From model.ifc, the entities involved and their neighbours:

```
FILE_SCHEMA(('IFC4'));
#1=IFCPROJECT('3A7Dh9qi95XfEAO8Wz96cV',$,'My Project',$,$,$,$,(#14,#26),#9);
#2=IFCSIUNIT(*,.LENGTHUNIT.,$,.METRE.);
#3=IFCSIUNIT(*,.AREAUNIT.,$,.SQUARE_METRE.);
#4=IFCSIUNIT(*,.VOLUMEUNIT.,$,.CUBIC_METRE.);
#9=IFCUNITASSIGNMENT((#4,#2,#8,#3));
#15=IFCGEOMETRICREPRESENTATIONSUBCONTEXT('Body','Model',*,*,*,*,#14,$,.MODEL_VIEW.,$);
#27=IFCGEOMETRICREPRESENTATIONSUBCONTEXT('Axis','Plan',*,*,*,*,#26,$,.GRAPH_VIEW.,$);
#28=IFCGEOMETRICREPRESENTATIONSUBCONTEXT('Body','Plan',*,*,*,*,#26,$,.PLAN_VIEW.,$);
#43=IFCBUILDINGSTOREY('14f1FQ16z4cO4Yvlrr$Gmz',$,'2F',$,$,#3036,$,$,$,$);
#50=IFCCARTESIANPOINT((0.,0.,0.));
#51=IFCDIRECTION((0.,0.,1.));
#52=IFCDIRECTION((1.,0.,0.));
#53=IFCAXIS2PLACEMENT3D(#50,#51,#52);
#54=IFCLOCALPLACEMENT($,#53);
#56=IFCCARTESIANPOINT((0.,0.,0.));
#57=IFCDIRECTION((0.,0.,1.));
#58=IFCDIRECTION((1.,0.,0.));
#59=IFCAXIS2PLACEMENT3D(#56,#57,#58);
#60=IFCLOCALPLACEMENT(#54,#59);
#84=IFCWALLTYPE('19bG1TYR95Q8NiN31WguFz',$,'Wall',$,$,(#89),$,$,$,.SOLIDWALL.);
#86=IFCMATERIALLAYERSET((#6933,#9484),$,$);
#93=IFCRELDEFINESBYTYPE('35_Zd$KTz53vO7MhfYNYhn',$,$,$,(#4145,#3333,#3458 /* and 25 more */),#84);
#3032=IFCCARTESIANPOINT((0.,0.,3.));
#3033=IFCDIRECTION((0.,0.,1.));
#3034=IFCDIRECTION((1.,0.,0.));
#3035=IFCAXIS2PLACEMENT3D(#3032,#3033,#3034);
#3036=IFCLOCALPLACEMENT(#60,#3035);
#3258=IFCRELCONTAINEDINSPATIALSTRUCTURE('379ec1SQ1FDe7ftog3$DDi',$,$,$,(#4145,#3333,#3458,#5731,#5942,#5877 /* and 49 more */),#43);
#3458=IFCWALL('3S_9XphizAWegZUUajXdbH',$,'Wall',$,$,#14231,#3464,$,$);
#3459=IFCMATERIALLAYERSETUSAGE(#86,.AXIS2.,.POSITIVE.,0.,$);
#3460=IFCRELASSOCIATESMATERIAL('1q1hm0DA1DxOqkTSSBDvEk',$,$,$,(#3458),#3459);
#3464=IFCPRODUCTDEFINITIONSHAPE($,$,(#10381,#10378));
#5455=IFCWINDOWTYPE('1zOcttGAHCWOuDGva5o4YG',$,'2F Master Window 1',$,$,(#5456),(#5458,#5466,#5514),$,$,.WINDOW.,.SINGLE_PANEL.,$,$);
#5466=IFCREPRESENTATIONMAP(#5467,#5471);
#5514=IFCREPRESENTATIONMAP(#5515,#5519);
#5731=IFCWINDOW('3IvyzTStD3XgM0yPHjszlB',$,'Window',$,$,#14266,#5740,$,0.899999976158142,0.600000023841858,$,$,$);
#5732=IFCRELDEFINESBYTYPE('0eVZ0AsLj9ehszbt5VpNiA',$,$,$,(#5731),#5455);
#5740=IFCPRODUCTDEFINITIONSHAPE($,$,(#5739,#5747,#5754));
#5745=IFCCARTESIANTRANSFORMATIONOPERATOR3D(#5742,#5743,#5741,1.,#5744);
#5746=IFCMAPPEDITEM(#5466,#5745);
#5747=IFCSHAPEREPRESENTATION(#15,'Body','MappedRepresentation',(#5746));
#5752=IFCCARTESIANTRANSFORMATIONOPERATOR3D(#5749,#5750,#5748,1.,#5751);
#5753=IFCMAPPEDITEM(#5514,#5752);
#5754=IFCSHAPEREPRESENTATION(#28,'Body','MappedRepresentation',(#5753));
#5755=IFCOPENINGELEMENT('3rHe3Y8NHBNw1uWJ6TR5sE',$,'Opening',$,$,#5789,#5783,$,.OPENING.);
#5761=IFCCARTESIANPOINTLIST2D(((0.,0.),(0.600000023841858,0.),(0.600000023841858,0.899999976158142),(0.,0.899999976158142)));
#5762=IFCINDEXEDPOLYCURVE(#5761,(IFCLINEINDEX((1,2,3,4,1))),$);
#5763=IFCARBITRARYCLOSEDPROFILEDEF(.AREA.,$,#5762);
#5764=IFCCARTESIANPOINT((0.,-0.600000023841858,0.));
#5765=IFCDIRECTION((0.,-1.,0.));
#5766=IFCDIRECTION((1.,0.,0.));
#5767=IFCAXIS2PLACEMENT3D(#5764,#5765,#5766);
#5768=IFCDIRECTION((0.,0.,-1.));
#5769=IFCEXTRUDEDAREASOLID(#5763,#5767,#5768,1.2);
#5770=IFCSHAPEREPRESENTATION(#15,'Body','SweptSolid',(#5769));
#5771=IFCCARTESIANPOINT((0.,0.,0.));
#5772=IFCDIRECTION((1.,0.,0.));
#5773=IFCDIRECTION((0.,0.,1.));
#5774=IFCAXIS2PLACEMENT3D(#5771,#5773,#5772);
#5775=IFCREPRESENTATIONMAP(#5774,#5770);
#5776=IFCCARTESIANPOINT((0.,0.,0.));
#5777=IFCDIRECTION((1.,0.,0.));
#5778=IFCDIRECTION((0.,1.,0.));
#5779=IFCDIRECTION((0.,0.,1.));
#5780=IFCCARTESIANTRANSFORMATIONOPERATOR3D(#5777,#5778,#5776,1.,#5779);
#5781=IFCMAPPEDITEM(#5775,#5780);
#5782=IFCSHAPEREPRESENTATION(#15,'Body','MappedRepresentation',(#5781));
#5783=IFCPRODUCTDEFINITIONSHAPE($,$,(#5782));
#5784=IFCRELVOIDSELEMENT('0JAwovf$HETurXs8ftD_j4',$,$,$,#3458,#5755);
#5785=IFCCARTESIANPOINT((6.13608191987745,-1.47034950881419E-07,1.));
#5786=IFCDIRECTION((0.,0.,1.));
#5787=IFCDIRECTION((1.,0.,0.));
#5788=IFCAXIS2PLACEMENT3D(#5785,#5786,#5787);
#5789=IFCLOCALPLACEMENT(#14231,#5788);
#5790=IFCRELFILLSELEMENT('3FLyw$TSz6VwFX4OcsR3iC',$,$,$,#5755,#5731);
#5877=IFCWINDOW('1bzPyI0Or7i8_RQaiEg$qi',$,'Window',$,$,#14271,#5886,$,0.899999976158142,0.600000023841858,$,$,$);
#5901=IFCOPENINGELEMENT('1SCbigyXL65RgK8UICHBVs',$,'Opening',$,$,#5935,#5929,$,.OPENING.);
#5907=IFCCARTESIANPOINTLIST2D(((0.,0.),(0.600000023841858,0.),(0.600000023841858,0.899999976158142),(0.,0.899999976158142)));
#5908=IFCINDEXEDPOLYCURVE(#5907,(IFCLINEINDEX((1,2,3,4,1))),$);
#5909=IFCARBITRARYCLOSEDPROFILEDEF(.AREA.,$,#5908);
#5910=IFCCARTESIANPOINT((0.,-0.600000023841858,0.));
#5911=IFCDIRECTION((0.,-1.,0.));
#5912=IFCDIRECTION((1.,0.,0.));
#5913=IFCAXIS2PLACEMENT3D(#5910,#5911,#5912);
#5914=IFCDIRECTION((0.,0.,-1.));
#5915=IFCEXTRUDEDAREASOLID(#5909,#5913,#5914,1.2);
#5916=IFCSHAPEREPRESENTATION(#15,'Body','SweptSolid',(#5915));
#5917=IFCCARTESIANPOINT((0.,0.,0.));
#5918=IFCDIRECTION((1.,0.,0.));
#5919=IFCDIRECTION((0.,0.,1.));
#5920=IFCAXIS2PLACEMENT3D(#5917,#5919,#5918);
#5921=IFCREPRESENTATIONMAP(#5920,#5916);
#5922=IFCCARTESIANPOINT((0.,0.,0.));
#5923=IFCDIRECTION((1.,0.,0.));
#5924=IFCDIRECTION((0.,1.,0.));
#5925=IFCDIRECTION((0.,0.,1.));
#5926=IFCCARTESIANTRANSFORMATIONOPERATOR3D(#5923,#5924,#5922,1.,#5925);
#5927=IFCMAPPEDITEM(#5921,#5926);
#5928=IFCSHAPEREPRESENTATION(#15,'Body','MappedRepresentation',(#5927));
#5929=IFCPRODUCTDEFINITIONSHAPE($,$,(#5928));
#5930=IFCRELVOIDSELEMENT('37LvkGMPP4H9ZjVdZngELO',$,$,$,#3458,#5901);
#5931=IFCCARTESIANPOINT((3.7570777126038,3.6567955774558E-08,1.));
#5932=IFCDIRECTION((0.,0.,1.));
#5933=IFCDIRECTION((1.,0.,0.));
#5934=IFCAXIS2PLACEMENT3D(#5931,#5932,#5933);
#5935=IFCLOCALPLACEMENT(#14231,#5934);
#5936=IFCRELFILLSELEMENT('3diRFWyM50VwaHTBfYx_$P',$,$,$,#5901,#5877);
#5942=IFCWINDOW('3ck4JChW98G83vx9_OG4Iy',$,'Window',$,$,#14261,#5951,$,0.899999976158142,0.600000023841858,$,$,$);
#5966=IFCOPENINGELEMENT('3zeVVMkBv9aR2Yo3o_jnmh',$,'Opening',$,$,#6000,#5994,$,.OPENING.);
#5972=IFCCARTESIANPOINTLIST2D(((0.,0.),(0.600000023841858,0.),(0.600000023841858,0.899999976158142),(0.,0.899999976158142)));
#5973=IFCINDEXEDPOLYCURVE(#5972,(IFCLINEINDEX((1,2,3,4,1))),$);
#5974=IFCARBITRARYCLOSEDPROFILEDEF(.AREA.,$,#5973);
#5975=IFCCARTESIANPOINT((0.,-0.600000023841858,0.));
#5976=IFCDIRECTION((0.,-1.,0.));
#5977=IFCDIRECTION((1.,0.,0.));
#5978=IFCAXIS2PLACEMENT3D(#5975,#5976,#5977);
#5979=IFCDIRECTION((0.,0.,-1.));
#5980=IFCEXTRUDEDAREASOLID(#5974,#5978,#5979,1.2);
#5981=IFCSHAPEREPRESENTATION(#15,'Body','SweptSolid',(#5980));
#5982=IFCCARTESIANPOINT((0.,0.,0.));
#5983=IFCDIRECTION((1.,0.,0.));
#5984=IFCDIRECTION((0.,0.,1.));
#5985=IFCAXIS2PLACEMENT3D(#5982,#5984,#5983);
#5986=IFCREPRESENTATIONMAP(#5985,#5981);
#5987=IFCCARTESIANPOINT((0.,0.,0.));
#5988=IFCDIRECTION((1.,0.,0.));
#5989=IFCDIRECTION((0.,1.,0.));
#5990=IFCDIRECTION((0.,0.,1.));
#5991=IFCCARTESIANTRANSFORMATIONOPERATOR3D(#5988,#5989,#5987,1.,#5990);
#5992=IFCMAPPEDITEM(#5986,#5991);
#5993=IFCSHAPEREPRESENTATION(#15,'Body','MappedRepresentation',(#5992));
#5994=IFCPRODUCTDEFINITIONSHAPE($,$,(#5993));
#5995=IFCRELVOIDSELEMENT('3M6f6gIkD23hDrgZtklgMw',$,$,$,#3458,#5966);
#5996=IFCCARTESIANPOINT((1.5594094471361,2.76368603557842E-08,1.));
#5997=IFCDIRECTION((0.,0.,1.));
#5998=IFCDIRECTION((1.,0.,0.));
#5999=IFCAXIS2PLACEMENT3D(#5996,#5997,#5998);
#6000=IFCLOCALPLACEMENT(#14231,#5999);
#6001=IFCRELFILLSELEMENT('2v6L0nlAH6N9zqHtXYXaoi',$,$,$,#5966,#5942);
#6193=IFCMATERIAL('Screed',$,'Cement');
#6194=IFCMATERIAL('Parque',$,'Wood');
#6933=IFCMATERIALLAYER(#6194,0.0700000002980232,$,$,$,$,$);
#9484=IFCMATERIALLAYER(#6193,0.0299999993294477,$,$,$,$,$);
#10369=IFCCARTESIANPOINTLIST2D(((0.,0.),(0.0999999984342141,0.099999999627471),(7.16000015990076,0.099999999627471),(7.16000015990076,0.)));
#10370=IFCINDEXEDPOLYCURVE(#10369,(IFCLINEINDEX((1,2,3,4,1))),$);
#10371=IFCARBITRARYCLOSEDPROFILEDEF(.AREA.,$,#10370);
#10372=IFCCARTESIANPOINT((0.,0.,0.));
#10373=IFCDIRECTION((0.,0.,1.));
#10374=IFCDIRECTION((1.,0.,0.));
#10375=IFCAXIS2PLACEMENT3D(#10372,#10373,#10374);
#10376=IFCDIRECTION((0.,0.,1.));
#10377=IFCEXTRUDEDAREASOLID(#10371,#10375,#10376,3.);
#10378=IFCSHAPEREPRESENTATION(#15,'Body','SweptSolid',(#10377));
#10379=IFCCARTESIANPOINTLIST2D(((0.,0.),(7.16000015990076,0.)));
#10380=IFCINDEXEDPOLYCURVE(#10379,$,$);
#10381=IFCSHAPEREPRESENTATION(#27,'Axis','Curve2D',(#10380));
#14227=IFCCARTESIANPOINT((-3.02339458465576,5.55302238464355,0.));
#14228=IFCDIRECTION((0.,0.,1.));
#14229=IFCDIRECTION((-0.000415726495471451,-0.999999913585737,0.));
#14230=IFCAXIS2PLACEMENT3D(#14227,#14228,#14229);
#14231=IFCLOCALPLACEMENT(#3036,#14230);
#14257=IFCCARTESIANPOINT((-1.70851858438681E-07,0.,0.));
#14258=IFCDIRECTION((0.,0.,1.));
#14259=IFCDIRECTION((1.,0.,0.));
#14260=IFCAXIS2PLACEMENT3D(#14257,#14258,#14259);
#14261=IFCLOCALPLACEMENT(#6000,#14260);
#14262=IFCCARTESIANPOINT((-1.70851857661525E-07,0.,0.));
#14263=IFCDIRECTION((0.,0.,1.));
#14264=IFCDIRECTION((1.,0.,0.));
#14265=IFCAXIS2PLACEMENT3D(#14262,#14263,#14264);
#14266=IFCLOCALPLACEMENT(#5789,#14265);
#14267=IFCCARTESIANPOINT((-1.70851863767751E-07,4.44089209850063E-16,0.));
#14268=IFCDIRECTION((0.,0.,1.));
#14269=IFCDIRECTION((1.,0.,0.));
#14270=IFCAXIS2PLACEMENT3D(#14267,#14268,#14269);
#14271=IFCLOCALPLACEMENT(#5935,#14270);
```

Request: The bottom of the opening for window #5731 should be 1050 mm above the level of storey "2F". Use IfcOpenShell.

```python
import numpy as np
import ifcopenshell
import ifcopenshell.api.geometry
import ifcopenshell.geom
import ifcopenshell.util.element
import ifcopenshell.util.placement
import ifcopenshell.util.shape
import ifcopenshell.util.unit

model = ifcopenshell.open("model.ifc")
unit_scale = ifcopenshell.util.unit.calculate_unit_scale(model)

window = model.by_guid("3IvyzTStD3XgM0yPHjszlB")
opening = window.FillsVoids[0].RelatingOpeningElement
storey = ifcopenshell.util.element.get_container(window, ifc_class="IfcBuildingStorey")
level = ifcopenshell.util.placement.get_local_placement(storey.ObjectPlacement)[2, 3]

# The opening's origin need not be at the sill, so measure its lowest point.
shape = ifcopenshell.geom.create_shape(ifcopenshell.geom.settings(), opening)
bottom = ifcopenshell.util.shape.get_shape_bottom_elevation(shape, shape.geometry) / unit_scale
dz = level + 1.05 - bottom

shift = np.array([0.0, 0.0, dz])
# The window is placed relative to its opening, so it follows when the opening moves.
matrix = ifcopenshell.util.placement.get_local_placement(opening.ObjectPlacement)
matrix[:3, 3] += shift
ifcopenshell.api.geometry.edit_object_placement(
    model, product=opening, matrix=matrix, is_si=False, should_transform_children=True
)

print(f"moved by {dz * unit_scale:+.3f} m")

model.write("model_v2.ifc")
```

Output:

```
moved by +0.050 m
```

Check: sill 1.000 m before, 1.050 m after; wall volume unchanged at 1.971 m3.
